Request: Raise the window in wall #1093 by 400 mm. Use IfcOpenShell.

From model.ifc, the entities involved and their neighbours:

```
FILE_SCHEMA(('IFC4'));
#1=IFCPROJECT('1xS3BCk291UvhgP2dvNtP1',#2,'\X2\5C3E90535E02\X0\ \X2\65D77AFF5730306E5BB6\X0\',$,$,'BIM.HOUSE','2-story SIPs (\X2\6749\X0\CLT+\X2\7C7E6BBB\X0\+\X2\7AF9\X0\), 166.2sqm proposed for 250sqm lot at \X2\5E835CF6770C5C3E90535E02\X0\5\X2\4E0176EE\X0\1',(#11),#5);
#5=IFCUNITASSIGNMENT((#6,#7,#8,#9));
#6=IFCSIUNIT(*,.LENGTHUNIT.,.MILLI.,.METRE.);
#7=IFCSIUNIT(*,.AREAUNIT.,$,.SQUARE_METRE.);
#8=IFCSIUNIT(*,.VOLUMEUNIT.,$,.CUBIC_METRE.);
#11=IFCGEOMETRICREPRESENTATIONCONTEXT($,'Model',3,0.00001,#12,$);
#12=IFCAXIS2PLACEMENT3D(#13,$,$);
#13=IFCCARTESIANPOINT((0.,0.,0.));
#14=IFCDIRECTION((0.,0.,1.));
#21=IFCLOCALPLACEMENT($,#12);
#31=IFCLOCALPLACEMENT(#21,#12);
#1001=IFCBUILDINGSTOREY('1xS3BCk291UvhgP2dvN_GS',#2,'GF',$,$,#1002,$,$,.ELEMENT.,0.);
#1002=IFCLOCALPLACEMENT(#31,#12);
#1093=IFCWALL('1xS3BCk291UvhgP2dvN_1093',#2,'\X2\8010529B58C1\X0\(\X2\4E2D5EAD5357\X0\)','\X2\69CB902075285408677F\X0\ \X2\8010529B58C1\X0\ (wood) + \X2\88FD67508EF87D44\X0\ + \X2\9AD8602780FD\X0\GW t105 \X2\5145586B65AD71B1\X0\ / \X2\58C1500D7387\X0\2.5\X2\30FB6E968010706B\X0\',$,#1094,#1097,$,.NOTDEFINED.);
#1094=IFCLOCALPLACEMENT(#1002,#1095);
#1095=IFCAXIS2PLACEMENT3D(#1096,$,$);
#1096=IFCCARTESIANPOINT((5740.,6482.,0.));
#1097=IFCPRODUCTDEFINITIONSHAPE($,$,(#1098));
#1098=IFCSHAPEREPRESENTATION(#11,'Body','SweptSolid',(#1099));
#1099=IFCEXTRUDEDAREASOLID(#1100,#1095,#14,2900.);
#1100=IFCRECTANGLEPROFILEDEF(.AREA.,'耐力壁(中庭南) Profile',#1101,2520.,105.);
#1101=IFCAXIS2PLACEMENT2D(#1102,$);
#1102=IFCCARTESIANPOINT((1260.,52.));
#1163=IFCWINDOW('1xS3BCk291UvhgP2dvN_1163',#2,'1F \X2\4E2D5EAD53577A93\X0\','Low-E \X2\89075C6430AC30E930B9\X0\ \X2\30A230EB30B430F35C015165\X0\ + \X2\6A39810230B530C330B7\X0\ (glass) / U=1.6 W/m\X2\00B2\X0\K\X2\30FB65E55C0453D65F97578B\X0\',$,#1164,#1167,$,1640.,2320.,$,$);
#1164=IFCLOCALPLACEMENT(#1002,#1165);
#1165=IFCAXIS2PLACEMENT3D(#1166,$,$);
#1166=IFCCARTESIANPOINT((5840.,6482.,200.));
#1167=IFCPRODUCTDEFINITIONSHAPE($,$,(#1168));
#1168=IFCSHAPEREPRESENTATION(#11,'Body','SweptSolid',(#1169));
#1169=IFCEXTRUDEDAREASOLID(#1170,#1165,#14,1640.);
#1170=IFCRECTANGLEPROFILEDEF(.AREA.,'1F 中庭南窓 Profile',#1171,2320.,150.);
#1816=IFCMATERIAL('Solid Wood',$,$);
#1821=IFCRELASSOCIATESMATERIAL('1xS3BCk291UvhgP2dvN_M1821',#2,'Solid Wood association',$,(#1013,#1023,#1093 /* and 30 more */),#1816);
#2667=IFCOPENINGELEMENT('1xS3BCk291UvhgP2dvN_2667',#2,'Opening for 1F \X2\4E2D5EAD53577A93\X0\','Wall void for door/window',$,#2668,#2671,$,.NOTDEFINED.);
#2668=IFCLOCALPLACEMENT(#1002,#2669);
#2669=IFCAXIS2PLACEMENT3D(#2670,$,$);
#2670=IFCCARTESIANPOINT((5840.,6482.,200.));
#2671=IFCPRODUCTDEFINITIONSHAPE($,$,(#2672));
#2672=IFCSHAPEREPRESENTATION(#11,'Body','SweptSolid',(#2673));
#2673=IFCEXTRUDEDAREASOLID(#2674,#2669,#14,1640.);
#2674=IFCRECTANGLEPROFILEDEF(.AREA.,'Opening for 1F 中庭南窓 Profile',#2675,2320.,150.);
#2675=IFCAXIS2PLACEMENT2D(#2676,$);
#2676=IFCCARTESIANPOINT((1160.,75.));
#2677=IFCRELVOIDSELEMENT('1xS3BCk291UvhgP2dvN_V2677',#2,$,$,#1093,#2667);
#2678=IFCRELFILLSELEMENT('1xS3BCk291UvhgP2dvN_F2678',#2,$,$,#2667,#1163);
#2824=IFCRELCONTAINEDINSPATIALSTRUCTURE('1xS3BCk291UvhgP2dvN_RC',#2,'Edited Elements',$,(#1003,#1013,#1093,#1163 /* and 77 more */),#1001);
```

```python
import numpy as np
import ifcopenshell
import ifcopenshell.api.geometry
import ifcopenshell.util.placement
import ifcopenshell.util.unit

model = ifcopenshell.open("model.ifc")
unit_scale = ifcopenshell.util.unit.calculate_unit_scale(model)

window = model.by_guid("1xS3BCk291UvhgP2dvN_1163")
opening = window.FillsVoids[0].RelatingOpeningElement
dz = 0.4 / unit_scale

shift = np.array([0.0, 0.0, dz])
# The window is not placed relative to its opening, so move both.
for product in (opening, window):
    matrix = ifcopenshell.util.placement.get_local_placement(product.ObjectPlacement)
    matrix[:3, 3] += shift
    ifcopenshell.api.geometry.edit_object_placement(model, product=product, matrix=matrix, is_si=False)

print(f"moved by {dz * unit_scale:+.3f} m")

model.write("model_updated.ifc")
```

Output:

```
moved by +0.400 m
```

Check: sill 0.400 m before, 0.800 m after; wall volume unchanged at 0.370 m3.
